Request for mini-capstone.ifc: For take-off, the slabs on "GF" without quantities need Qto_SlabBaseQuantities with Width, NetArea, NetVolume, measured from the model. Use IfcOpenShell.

First a look at what the model holds.

```python
import ifcopenshell
import ifcopenshell.util.element
import ifcopenshell.util.unit

model = ifcopenshell.open("mini-capstone.ifc")
print(model.schema)
for unit_type in ("LENGTHUNIT", "AREAUNIT", "VOLUMEUNIT"):
    print(unit_type, ifcopenshell.util.unit.calculate_unit_scale(model, unit_type))
storey = next(s for s in model.by_type("IfcBuildingStorey") if s.Name == "GF")
slabs = [e for e in ifcopenshell.util.element.get_decomposition(storey) if e.is_a("IfcSlab")]
for e in sorted(slabs, key=lambda e: e.id()):
    print(e.id(), e.is_a(), e.Name, list(ifcopenshell.util.element.get_psets(e, qtos_only=True)), sep=" | ")
```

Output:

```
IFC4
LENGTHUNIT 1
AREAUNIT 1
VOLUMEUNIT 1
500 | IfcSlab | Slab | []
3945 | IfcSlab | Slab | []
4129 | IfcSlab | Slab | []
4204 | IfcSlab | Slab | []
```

```python
import ifcopenshell
import ifcopenshell.api.pset
import ifcopenshell.geom
import ifcopenshell.util.element
import ifcopenshell.util.shape
import ifcopenshell.util.unit

model = ifcopenshell.open("mini-capstone.ifc")
unit_scale = ifcopenshell.util.unit.calculate_unit_scale(model)
area_scale = ifcopenshell.util.unit.calculate_unit_scale(model, "AREAUNIT")
volume_scale = ifcopenshell.util.unit.calculate_unit_scale(model, "VOLUMEUNIT")
settings = ifcopenshell.geom.settings()

storey = next(s for s in model.by_type("IfcBuildingStorey") if s.Name == "GF")
slabs = [e for e in ifcopenshell.util.element.get_decomposition(storey) if e.is_a("IfcSlab")]

for e in sorted(slabs, key=lambda e: e.id()):
    if ifcopenshell.util.element.get_psets(e, qtos_only=True, should_inherit=False):
        continue
    # Geometry comes back in metres, in the element's own axes.
    shape = ifcopenshell.geom.create_shape(settings, e)
    values = {
        "Width": ifcopenshell.util.shape.get_z(shape.geometry) / unit_scale,
        "NetArea": ifcopenshell.util.shape.get_footprint_area(shape.geometry) / area_scale,
        "NetVolume": ifcopenshell.util.shape.get_volume(shape.geometry) / volume_scale,
    }
    qto = ifcopenshell.api.pset.add_qto(model, product=e, name="Qto_SlabBaseQuantities")
    ifcopenshell.api.pset.edit_qto(model, qto=qto, properties=values)
    print(e.id(), {k: round(v, 3) for k, v in values.items()})

model.write("mini-capstone_v2.ifc")
```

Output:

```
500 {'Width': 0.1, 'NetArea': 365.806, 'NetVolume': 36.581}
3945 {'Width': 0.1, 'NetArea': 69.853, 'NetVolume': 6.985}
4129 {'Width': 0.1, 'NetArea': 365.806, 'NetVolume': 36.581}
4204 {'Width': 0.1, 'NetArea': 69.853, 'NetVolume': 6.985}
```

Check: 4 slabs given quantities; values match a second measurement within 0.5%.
